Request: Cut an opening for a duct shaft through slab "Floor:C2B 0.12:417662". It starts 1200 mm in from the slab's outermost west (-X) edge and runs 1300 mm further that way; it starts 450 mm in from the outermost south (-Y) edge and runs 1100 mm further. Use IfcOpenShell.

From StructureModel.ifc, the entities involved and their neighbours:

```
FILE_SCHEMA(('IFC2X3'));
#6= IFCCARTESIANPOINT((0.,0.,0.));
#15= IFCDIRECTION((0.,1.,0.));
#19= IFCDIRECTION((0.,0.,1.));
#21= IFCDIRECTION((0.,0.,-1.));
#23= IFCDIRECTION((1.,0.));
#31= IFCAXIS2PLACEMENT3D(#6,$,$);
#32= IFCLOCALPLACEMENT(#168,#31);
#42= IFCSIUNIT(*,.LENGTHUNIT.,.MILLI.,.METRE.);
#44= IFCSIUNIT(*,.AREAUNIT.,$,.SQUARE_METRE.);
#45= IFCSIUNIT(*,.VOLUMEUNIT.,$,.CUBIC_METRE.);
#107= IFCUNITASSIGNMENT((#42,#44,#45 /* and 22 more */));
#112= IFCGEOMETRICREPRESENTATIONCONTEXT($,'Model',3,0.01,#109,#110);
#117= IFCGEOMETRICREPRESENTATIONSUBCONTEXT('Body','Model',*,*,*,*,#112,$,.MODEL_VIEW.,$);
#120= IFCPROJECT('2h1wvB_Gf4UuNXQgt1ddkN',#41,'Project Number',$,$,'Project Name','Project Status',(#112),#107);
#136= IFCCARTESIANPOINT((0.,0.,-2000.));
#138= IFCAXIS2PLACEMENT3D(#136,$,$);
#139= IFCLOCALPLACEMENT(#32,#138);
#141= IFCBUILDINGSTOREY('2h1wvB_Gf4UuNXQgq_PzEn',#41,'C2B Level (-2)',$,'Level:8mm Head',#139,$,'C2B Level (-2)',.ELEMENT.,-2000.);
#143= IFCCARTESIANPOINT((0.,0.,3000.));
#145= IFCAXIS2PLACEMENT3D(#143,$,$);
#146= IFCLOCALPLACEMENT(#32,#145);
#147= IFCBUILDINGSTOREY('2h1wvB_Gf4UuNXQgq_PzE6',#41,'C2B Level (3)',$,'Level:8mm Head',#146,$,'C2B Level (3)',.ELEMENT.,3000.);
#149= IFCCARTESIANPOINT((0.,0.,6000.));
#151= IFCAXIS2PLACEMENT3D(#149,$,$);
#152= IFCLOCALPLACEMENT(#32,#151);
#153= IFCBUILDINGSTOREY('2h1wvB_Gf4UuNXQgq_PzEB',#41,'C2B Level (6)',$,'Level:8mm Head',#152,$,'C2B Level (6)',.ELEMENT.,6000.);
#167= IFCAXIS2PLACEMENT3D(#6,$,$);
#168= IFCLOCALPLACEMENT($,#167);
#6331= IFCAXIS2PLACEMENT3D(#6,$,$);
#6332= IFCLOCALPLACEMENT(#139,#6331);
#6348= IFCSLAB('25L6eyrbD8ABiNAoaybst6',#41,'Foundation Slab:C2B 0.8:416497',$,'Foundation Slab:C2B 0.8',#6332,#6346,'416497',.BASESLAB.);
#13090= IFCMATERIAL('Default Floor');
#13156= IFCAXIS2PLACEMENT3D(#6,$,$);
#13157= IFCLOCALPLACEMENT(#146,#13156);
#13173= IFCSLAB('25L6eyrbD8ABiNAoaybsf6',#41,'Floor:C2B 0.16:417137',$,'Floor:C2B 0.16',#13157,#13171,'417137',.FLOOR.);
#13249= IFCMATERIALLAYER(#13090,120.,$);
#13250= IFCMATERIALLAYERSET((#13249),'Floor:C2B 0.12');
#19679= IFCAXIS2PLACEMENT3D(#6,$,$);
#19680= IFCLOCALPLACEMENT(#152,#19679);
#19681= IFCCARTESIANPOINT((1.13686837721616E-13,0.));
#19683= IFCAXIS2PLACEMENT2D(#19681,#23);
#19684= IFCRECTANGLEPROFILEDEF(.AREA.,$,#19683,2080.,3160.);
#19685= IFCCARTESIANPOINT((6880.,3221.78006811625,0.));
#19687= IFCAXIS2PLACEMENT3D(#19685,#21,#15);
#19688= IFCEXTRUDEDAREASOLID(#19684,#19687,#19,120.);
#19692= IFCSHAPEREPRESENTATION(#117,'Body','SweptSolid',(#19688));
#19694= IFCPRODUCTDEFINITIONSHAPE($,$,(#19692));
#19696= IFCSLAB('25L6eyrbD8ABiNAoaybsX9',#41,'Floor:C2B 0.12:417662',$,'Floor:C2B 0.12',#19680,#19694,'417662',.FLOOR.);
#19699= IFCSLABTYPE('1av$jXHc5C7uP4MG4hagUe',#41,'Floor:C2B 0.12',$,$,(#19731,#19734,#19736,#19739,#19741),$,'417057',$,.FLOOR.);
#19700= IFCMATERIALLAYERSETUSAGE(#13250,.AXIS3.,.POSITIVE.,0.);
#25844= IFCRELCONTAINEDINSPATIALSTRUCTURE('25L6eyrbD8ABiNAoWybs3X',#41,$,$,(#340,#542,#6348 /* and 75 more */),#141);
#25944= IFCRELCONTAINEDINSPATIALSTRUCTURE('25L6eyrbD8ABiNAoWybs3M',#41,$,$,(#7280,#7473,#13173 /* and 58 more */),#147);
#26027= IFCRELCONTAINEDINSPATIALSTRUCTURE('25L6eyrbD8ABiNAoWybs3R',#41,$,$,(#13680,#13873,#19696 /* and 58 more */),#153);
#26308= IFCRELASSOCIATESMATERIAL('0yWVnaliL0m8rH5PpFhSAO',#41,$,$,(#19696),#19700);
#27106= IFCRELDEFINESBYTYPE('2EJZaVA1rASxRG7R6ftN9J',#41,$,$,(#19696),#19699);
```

```python
import numpy as np
import ifcopenshell
import ifcopenshell.api.feature
import ifcopenshell.api.geometry
import ifcopenshell.api.root
import ifcopenshell.geom
import ifcopenshell.util.placement
import ifcopenshell.util.representation
import ifcopenshell.util.shape
import ifcopenshell.util.unit

model = ifcopenshell.open("StructureModel.ifc")
unit_scale = ifcopenshell.util.unit.calculate_unit_scale(model)
settings = ifcopenshell.geom.settings()


def volume(element):
    """Net volume in cubic metres, openings subtracted."""
    shape = ifcopenshell.geom.create_shape(settings, element)
    return ifcopenshell.util.shape.get_volume(shape.geometry)


slab = model.by_guid("25L6eyrbD8ABiNAoaybsX9")
before = volume(slab)

# Extent in the slab's own axes, in metres. The edges named are its -X and -Y sides.
slab_shape = ifcopenshell.geom.create_shape(settings, slab)
vertices = ifcopenshell.util.shape.get_vertices(slab_shape.geometry)
x_min, y_min, bottom = vertices.min(axis=0)
top = vertices[:, 2].max()

opening = ifcopenshell.api.root.create_entity(model, ifc_class="IfcOpeningElement", name="Duct shaft opening")
context = ifcopenshell.util.representation.get_context(model, "Model", "Body", "MODEL_VIEW")
width, depth = 1.3, 1.1
outline = [(0.0, 0.0), (width, 0.0), (width, depth), (0.0, depth), (0.0, 0.0)]
# Overshoot both faces by 50 mm so the cut is clean.
shape = ifcopenshell.api.geometry.add_slab_representation(
    model, context=context, depth=top - bottom + 0.1, polyline=outline
)
ifcopenshell.api.geometry.assign_representation(model, product=opening, representation=shape)

matrix = ifcopenshell.util.placement.get_local_placement(slab.ObjectPlacement)
matrix[:, 3] = matrix @ np.append(np.array([x_min + 1.2, y_min + 0.45, bottom - 0.05]) / unit_scale, 1.0)
ifcopenshell.api.geometry.edit_object_placement(model, product=opening, matrix=matrix, is_si=False)
ifcopenshell.api.feature.add_feature(model, feature=opening, element=slab)

after = volume(slab)

print(f"slab volume {before:.3f} -> {after:.3f} m3")

model.write("StructureModel_updated.ifc")
```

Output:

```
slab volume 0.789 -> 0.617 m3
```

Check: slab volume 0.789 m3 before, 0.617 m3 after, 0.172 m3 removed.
